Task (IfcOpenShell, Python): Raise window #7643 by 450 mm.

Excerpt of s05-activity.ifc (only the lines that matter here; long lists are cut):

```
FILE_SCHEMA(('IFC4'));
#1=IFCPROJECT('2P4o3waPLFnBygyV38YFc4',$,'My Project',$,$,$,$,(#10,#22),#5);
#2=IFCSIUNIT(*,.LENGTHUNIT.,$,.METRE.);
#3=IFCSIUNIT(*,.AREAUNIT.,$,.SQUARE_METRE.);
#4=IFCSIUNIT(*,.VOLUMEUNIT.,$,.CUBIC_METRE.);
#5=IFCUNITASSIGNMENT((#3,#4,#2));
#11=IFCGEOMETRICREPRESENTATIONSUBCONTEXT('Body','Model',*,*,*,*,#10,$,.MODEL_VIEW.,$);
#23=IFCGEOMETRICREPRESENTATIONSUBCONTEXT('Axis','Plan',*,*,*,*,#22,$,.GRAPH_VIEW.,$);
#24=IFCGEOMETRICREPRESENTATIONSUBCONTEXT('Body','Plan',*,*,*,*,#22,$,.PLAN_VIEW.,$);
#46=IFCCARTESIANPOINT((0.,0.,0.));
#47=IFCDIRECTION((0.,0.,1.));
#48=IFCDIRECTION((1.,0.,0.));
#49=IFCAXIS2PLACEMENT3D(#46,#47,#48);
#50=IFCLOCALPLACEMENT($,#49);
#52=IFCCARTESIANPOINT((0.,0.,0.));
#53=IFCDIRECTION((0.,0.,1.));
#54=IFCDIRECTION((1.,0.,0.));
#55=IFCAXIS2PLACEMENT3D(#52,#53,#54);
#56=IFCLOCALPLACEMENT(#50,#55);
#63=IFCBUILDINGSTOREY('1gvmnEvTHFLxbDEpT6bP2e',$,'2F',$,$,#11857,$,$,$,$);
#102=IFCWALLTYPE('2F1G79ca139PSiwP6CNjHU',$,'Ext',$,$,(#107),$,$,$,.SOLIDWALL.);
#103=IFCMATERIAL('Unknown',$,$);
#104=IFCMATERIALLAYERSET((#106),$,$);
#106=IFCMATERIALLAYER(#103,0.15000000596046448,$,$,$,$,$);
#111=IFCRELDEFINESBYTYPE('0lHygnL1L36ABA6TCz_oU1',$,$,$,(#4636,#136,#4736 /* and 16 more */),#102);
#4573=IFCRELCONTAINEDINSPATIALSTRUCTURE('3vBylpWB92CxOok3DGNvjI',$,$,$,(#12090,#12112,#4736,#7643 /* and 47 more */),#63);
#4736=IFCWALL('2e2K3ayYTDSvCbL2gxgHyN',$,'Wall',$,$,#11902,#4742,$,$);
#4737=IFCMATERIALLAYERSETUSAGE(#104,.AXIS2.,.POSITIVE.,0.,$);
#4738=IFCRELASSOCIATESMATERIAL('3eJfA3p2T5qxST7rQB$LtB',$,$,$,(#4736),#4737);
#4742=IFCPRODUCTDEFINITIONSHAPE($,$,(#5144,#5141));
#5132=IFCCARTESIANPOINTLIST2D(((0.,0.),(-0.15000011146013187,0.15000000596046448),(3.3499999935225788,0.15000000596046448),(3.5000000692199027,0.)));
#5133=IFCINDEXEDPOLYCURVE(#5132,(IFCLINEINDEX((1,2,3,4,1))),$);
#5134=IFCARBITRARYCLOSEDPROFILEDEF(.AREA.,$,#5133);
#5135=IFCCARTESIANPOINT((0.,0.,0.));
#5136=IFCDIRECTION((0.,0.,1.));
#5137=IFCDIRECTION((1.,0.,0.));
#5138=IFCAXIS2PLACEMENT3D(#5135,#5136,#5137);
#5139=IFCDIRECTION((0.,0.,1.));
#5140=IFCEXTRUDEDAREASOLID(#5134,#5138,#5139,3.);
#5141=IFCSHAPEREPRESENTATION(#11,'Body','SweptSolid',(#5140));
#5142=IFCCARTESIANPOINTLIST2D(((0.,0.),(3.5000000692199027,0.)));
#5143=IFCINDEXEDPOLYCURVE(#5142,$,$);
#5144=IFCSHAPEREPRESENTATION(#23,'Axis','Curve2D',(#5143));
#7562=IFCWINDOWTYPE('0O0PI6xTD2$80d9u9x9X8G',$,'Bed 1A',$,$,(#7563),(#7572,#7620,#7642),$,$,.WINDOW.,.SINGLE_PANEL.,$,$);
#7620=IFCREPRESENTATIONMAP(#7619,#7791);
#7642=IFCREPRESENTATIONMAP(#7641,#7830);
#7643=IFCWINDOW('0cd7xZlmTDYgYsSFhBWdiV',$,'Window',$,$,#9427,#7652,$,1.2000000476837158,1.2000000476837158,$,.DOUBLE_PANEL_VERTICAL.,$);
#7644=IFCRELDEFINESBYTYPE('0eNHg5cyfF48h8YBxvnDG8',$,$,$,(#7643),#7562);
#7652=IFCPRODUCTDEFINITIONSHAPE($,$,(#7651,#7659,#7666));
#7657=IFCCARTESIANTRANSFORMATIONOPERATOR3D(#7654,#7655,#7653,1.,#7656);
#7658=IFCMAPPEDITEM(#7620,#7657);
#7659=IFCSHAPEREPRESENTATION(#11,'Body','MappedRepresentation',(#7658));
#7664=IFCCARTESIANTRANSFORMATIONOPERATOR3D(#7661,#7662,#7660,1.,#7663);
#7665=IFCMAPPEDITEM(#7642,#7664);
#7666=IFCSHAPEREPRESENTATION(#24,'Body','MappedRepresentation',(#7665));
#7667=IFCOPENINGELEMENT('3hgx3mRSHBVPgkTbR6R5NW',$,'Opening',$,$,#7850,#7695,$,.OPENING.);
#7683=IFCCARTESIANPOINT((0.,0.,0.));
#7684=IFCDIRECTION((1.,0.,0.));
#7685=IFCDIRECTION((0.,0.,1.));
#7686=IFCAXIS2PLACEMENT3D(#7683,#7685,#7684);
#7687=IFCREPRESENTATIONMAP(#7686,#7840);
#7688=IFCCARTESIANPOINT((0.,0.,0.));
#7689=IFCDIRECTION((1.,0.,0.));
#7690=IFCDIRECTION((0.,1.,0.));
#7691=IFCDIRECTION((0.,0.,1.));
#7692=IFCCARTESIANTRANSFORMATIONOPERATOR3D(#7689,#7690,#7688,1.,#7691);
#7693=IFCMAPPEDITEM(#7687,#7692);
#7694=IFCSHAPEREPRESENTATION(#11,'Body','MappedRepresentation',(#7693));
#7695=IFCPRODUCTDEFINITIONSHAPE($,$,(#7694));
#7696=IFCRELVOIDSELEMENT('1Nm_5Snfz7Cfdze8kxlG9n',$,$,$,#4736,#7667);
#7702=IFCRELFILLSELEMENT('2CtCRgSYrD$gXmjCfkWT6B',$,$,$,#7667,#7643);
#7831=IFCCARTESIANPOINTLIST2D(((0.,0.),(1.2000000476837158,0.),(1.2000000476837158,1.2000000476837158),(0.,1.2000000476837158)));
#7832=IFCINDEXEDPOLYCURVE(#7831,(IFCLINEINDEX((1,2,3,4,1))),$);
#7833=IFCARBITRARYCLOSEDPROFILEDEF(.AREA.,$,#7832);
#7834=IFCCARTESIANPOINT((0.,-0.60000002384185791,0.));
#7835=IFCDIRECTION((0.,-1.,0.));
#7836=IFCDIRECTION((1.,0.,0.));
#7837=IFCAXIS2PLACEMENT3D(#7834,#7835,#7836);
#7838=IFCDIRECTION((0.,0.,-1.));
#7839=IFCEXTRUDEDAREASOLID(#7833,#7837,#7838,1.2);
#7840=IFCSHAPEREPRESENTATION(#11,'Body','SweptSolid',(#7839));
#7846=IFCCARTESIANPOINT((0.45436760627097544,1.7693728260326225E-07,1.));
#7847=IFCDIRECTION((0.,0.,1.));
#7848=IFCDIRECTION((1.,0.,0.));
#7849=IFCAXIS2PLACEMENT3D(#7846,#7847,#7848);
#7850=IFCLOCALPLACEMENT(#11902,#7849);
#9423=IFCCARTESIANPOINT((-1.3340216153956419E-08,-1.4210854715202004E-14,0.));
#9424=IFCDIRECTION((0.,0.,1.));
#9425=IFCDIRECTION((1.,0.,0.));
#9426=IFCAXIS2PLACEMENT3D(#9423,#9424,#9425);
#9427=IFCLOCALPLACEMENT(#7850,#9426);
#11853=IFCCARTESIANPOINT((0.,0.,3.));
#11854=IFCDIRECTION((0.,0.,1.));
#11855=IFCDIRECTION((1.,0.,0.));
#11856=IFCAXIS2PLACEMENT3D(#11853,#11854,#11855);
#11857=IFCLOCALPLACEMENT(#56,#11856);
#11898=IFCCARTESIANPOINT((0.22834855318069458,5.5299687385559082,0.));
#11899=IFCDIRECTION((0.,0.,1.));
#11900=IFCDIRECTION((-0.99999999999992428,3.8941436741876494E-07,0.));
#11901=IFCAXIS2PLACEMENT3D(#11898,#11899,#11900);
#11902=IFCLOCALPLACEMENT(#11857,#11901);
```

```python
import numpy as np
import ifcopenshell
import ifcopenshell.api.geometry
import ifcopenshell.util.placement
import ifcopenshell.util.unit

model = ifcopenshell.open("s05-activity.ifc")
unit_scale = ifcopenshell.util.unit.calculate_unit_scale(model)

window = model.by_id(7643)
opening = window.FillsVoids[0].RelatingOpeningElement
dz = 0.45

shift = np.array([0.0, 0.0, dz])
# The window is placed relative to its opening, so it follows when the opening moves.
matrix = ifcopenshell.util.placement.get_local_placement(opening.ObjectPlacement)
matrix[:3, 3] += shift
ifcopenshell.api.geometry.edit_object_placement(
    model, product=opening, matrix=matrix, is_si=False, should_transform_children=True
)

print(f"moved by {dz * unit_scale:+.3f} m")

model.write("s05-activity_v2.ifc")
```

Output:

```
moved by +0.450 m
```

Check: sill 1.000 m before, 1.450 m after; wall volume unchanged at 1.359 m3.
